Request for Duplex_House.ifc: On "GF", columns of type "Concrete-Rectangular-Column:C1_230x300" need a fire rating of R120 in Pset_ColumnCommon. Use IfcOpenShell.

First a look at what the model holds.

```python
import ifcopenshell
import ifcopenshell.util.element

model = ifcopenshell.open("Duplex_House.ifc")
print(model.schema)
storey = next(s for s in model.by_type("IfcBuildingStorey") if s.Name == "GF")
columns = [e for e in ifcopenshell.util.element.get_decomposition(storey) if e.is_a("IfcColumn")]
seen = {}
for e in columns:
    element_type = ifcopenshell.util.element.get_type(e)
    key = (element_type.Name if element_type != e and element_type else None, ifcopenshell.util.element.get_pset(e, "Pset_ColumnCommon", "FireRating"))
    seen[key] = seen.get(key, 0) + 1
for (name, value), count in sorted(seen.items(), key=str):
    print(count, "x", name, "|", value)
```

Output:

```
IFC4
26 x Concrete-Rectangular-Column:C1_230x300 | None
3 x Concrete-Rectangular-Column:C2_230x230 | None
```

```python
import ifcopenshell
import ifcopenshell.api.pset
import ifcopenshell.util.element

model = ifcopenshell.open("Duplex_House.ifc")

storey = next(s for s in model.by_type("IfcBuildingStorey") if s.Name == "GF")
columns = [e for e in ifcopenshell.util.element.get_decomposition(storey) if e.is_a("IfcColumn")]

count = 0
for e in columns:
    element_type = ifcopenshell.util.element.get_type(e)
    if element_type in (None, e) or element_type.Name != "Concrete-Rectangular-Column:C1_230x300":
        continue
    # add_pset returns the element's existing set when there is one.
    pset = ifcopenshell.api.pset.add_pset(model, product=e, name="Pset_ColumnCommon")
    ifcopenshell.api.pset.edit_pset(model, pset=pset, properties={"FireRating": "R120"})
    count += 1

print(count, "columns updated")

model.write("Duplex_House_updated.ifc")
```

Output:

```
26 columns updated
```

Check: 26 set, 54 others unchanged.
